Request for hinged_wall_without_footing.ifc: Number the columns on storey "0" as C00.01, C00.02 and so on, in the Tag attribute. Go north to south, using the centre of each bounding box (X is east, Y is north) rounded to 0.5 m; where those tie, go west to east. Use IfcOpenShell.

First a look at what the model holds.

```python
import ifcopenshell
import ifcopenshell.util.element
import ifcopenshell.util.placement

model = ifcopenshell.open("hinged_wall_without_footing.ifc")
print(model.schema)
storey = next(s for s in model.by_type("IfcBuildingStorey") if s.Name == "0")
columns = [e for e in ifcopenshell.util.element.get_decomposition(storey) if e.is_a("IfcColumn")]
for e in sorted(columns, key=lambda e: e.id()):
    origin = ifcopenshell.util.placement.get_local_placement(e.ObjectPlacement)[:3, 3]
    print(e.id(), e.Tag, e.Name, origin.round(2) + 0.0, sep=" | ")
```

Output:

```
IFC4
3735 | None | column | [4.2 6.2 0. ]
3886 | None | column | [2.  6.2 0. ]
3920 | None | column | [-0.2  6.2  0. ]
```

```python
import ifcopenshell
import ifcopenshell.geom
import ifcopenshell.util.element
import ifcopenshell.util.shape

model = ifcopenshell.open("hinged_wall_without_footing.ifc")
settings = ifcopenshell.geom.settings()
settings.set("use-world-coords", True)


def centre(element):
    shape = ifcopenshell.geom.create_shape(settings, element)
    return ifcopenshell.util.shape.get_bbox_centroid(shape.geometry)


storey = next(s for s in model.by_type("IfcBuildingStorey") if s.Name == "0")
columns = [e for e in ifcopenshell.util.element.get_decomposition(storey) if e.is_a("IfcColumn")]

# Insertion points can sit at a corner or the storey origin, so sort by the geometry (in metres).
centres = {e: centre(e) for e in columns}
columns.sort(key=lambda e: (-round(centres[e][1] / 0.5), centres[e][0]))

for i, e in enumerate(columns, start=1):
    number = f"C00.{i:02d}"
    e.Tag = number
    print(e.id(), number)

model.write("hinged_wall_without_footing_edited.ifc")
```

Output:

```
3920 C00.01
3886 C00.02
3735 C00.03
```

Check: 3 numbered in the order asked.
